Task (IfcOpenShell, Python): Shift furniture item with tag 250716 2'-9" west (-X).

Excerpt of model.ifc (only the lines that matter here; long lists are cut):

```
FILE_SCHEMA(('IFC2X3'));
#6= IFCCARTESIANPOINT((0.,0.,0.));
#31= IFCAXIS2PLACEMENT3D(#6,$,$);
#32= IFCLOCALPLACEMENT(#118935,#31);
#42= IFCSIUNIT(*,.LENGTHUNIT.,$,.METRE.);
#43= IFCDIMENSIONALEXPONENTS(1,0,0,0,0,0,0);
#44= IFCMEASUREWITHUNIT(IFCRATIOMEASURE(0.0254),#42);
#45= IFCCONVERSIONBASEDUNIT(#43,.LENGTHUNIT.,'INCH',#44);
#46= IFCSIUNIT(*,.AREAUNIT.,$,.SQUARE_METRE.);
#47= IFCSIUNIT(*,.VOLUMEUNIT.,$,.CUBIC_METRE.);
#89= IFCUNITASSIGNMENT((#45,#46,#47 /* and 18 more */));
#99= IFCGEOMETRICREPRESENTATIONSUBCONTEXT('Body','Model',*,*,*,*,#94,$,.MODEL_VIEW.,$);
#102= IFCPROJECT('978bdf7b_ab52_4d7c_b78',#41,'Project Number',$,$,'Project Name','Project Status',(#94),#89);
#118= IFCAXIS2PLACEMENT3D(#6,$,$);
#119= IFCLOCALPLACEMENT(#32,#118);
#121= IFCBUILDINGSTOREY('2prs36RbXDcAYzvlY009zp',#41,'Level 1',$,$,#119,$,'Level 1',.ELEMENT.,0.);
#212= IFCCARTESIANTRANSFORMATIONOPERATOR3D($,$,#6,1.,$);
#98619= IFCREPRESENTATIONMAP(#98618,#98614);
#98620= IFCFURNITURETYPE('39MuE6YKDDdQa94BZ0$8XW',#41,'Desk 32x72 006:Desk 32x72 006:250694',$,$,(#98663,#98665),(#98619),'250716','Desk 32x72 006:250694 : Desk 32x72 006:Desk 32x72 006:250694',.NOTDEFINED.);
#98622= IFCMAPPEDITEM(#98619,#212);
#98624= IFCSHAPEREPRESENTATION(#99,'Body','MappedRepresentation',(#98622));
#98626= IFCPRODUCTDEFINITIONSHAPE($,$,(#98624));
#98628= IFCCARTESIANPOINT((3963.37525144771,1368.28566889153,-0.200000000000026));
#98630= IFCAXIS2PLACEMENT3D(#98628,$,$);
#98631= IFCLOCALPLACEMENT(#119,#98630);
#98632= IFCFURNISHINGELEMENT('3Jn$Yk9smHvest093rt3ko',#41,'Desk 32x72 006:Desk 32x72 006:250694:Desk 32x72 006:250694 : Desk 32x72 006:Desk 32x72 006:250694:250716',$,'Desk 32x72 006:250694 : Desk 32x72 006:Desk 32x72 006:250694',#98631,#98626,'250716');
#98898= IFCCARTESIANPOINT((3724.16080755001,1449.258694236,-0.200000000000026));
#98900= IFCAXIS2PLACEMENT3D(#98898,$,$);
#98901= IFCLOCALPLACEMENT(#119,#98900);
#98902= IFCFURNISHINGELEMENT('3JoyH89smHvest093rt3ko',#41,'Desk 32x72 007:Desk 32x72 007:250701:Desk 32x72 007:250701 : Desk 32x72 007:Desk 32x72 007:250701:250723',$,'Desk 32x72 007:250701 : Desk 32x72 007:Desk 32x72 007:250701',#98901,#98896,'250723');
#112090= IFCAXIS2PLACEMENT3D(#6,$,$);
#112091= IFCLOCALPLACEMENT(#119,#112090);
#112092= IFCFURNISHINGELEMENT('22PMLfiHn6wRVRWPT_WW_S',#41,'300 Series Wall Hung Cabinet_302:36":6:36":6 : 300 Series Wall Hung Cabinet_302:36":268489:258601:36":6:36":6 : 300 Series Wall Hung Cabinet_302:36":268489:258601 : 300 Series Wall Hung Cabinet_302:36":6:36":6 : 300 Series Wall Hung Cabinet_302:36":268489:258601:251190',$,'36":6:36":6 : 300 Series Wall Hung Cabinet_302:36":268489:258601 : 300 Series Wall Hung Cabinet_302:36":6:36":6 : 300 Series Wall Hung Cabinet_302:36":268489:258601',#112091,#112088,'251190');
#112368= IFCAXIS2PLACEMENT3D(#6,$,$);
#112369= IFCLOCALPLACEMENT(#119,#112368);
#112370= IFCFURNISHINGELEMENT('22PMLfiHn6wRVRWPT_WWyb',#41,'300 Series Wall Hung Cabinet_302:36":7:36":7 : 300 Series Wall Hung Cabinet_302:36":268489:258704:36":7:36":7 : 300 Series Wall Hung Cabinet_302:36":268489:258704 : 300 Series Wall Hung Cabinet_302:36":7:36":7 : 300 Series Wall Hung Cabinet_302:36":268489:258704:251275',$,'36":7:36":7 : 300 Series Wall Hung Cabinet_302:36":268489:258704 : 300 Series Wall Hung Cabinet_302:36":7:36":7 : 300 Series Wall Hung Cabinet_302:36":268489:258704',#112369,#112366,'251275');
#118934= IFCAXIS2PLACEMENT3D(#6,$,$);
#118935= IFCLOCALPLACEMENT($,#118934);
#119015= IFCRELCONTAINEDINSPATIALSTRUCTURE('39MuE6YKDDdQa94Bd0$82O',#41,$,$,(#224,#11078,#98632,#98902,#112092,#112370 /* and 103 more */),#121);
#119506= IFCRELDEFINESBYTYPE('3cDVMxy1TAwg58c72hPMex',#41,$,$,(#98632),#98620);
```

```python
import ifcopenshell
import ifcopenshell.api.geometry
import ifcopenshell.util.placement
import ifcopenshell.util.unit

model = ifcopenshell.open("model.ifc")
unit_scale = ifcopenshell.util.unit.calculate_unit_scale(model)

item = model.by_guid("3Jn$Yk9smHvest093rt3ko")
matrix = ifcopenshell.util.placement.get_local_placement(item.ObjectPlacement)
matrix[0, 3] -= 33 * 0.0254 / unit_scale
ifcopenshell.api.geometry.edit_object_placement(model, product=item, matrix=matrix, is_si=False)

print(ifcopenshell.util.placement.get_local_placement(item.ObjectPlacement).round(3) + 0.0)

model.write("model_v2.ifc")
```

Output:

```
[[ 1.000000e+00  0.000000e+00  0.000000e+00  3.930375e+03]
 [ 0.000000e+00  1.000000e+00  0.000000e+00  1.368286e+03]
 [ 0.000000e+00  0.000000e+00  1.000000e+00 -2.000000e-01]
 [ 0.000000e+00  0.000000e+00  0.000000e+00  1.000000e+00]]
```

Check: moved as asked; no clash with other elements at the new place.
